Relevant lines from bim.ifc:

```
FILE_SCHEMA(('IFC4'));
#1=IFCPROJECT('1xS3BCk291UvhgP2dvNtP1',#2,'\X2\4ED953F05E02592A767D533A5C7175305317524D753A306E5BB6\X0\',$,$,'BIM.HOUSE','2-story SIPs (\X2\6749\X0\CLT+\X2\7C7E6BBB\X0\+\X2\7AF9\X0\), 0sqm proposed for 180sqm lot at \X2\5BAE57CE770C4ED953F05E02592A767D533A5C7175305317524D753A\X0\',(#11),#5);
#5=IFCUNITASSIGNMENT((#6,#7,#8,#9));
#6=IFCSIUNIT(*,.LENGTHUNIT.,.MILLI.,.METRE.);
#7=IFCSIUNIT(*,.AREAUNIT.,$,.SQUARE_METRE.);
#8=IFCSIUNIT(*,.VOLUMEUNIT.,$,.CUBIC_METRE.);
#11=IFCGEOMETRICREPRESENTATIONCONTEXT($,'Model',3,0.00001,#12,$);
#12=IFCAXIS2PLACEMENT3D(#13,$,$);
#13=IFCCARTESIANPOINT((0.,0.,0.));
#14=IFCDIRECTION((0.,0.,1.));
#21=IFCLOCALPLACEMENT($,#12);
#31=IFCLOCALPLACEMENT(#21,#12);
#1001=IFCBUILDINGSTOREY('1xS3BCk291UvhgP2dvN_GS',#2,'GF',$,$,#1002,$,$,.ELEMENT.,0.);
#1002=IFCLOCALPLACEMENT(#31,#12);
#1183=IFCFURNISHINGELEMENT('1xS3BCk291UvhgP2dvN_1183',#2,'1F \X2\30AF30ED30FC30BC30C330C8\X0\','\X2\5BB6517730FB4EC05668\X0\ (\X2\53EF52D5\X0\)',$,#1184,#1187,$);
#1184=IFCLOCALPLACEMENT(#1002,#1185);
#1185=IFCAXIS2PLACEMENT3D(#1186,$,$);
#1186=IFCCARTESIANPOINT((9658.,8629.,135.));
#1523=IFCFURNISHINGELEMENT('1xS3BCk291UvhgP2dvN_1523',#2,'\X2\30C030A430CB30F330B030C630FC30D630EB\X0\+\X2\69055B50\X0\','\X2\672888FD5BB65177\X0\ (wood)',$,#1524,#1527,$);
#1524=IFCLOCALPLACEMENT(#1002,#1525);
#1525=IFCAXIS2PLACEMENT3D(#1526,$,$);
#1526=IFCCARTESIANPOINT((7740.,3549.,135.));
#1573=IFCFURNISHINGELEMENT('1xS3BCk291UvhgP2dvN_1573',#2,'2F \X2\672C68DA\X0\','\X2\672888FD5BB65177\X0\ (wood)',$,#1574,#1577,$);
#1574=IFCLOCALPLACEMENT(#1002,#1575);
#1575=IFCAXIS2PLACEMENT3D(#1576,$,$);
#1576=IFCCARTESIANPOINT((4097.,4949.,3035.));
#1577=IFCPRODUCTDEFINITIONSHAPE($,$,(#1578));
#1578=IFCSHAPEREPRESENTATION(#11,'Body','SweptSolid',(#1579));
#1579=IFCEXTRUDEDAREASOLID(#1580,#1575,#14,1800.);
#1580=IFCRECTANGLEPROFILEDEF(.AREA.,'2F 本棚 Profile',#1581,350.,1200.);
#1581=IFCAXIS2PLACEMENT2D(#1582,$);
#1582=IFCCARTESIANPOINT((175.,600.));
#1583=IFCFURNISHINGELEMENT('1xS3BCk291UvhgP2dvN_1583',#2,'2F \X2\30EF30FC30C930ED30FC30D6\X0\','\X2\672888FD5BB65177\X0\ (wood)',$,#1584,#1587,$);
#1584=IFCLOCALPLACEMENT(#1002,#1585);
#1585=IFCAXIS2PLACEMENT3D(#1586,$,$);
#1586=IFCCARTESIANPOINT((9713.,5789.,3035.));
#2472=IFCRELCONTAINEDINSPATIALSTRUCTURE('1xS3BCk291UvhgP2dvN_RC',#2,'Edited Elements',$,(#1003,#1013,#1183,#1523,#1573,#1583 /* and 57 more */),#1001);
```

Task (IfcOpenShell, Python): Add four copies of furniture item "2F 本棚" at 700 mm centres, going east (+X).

```python
import numpy as np
import ifcopenshell
import ifcopenshell.api.geometry
import ifcopenshell.api.root
import ifcopenshell.util.element
import ifcopenshell.util.placement
import ifcopenshell.util.unit

model = ifcopenshell.open("bim.ifc")
unit_scale = ifcopenshell.util.unit.calculate_unit_scale(model)


def reuse_history(source, copy):
    """copy_class also copies each property set's owner history, people and application; keep the originals."""
    for rel in copy.IsDefinedBy:
        if rel.is_a("IfcRelDefinesByProperties") and (history := rel.RelatingPropertyDefinition.OwnerHistory):
            rel.RelatingPropertyDefinition.OwnerHistory = source.OwnerHistory
            ifcopenshell.util.element.remove_deep2(model, history)


source = model.by_id(1573)
base = ifcopenshell.util.placement.get_local_placement(source.ObjectPlacement)
step = np.array([1.0, 0.0, 0.0]) * 0.7 / unit_scale

for i in range(1, 5):
    copy = ifcopenshell.api.root.copy_class(model, product=source)
    copy.Representation = ifcopenshell.util.element.copy_deep(
        model, source.Representation, exclude=["IfcGeometricRepresentationContext", "IfcRepresentationMap"]
    )
    reuse_history(source, copy)
    matrix = base.copy()
    matrix[:3, 3] += i * step
    print("added at", matrix[:3, 3].round(3) + 0.0)
    ifcopenshell.api.geometry.edit_object_placement(model, product=copy, matrix=matrix, is_si=False)

model.write("bim_v2.ifc")
```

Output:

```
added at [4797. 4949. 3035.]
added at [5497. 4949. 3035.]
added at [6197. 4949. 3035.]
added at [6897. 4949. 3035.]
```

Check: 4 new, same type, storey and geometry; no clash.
